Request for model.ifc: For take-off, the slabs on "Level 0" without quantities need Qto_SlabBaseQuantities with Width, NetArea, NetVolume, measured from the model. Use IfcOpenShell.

First a look at what the model holds.

```python
import ifcopenshell
import ifcopenshell.util.element
import ifcopenshell.util.unit

model = ifcopenshell.open("model.ifc")
print(model.schema)
for unit_type in ("LENGTHUNIT", "AREAUNIT", "VOLUMEUNIT"):
    print(unit_type, ifcopenshell.util.unit.calculate_unit_scale(model, unit_type))
storey = next(s for s in model.by_type("IfcBuildingStorey") if s.Name == "Level 0")
slabs = [e for e in ifcopenshell.util.element.get_decomposition(storey) if e.is_a("IfcSlab")]
for e in sorted(slabs, key=lambda e: e.id()):
    print(e.id(), e.is_a(), e.Name, list(ifcopenshell.util.element.get_psets(e, qtos_only=True)), sep=" | ")
```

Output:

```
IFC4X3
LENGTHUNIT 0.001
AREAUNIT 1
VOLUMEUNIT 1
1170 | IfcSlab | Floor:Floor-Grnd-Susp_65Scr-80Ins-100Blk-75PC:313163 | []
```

```python
import ifcopenshell
import ifcopenshell.api.pset
import ifcopenshell.geom
import ifcopenshell.util.element
import ifcopenshell.util.shape
import ifcopenshell.util.unit

model = ifcopenshell.open("model.ifc")
unit_scale = ifcopenshell.util.unit.calculate_unit_scale(model)
area_scale = ifcopenshell.util.unit.calculate_unit_scale(model, "AREAUNIT")
volume_scale = ifcopenshell.util.unit.calculate_unit_scale(model, "VOLUMEUNIT")
settings = ifcopenshell.geom.settings()

storey = next(s for s in model.by_type("IfcBuildingStorey") if s.Name == "Level 0")
slabs = [e for e in ifcopenshell.util.element.get_decomposition(storey) if e.is_a("IfcSlab")]

for e in sorted(slabs, key=lambda e: e.id()):
    if ifcopenshell.util.element.get_psets(e, qtos_only=True, should_inherit=False):
        continue
    # Geometry comes back in metres, in the element's own axes.
    shape = ifcopenshell.geom.create_shape(settings, e)
    values = {
        "Width": ifcopenshell.util.shape.get_z(shape.geometry) / unit_scale,
        "NetArea": ifcopenshell.util.shape.get_footprint_area(shape.geometry) / area_scale,
        "NetVolume": ifcopenshell.util.shape.get_volume(shape.geometry) / volume_scale,
    }
    qto = ifcopenshell.api.pset.add_qto(model, product=e, name="Qto_SlabBaseQuantities")
    ifcopenshell.api.pset.edit_qto(model, qto=qto, properties=values)
    print(e.id(), {k: round(v, 3) for k, v in values.items()})

model.write("model-out.ifc")
```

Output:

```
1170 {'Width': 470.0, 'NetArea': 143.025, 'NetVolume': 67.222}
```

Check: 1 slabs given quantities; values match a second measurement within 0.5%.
